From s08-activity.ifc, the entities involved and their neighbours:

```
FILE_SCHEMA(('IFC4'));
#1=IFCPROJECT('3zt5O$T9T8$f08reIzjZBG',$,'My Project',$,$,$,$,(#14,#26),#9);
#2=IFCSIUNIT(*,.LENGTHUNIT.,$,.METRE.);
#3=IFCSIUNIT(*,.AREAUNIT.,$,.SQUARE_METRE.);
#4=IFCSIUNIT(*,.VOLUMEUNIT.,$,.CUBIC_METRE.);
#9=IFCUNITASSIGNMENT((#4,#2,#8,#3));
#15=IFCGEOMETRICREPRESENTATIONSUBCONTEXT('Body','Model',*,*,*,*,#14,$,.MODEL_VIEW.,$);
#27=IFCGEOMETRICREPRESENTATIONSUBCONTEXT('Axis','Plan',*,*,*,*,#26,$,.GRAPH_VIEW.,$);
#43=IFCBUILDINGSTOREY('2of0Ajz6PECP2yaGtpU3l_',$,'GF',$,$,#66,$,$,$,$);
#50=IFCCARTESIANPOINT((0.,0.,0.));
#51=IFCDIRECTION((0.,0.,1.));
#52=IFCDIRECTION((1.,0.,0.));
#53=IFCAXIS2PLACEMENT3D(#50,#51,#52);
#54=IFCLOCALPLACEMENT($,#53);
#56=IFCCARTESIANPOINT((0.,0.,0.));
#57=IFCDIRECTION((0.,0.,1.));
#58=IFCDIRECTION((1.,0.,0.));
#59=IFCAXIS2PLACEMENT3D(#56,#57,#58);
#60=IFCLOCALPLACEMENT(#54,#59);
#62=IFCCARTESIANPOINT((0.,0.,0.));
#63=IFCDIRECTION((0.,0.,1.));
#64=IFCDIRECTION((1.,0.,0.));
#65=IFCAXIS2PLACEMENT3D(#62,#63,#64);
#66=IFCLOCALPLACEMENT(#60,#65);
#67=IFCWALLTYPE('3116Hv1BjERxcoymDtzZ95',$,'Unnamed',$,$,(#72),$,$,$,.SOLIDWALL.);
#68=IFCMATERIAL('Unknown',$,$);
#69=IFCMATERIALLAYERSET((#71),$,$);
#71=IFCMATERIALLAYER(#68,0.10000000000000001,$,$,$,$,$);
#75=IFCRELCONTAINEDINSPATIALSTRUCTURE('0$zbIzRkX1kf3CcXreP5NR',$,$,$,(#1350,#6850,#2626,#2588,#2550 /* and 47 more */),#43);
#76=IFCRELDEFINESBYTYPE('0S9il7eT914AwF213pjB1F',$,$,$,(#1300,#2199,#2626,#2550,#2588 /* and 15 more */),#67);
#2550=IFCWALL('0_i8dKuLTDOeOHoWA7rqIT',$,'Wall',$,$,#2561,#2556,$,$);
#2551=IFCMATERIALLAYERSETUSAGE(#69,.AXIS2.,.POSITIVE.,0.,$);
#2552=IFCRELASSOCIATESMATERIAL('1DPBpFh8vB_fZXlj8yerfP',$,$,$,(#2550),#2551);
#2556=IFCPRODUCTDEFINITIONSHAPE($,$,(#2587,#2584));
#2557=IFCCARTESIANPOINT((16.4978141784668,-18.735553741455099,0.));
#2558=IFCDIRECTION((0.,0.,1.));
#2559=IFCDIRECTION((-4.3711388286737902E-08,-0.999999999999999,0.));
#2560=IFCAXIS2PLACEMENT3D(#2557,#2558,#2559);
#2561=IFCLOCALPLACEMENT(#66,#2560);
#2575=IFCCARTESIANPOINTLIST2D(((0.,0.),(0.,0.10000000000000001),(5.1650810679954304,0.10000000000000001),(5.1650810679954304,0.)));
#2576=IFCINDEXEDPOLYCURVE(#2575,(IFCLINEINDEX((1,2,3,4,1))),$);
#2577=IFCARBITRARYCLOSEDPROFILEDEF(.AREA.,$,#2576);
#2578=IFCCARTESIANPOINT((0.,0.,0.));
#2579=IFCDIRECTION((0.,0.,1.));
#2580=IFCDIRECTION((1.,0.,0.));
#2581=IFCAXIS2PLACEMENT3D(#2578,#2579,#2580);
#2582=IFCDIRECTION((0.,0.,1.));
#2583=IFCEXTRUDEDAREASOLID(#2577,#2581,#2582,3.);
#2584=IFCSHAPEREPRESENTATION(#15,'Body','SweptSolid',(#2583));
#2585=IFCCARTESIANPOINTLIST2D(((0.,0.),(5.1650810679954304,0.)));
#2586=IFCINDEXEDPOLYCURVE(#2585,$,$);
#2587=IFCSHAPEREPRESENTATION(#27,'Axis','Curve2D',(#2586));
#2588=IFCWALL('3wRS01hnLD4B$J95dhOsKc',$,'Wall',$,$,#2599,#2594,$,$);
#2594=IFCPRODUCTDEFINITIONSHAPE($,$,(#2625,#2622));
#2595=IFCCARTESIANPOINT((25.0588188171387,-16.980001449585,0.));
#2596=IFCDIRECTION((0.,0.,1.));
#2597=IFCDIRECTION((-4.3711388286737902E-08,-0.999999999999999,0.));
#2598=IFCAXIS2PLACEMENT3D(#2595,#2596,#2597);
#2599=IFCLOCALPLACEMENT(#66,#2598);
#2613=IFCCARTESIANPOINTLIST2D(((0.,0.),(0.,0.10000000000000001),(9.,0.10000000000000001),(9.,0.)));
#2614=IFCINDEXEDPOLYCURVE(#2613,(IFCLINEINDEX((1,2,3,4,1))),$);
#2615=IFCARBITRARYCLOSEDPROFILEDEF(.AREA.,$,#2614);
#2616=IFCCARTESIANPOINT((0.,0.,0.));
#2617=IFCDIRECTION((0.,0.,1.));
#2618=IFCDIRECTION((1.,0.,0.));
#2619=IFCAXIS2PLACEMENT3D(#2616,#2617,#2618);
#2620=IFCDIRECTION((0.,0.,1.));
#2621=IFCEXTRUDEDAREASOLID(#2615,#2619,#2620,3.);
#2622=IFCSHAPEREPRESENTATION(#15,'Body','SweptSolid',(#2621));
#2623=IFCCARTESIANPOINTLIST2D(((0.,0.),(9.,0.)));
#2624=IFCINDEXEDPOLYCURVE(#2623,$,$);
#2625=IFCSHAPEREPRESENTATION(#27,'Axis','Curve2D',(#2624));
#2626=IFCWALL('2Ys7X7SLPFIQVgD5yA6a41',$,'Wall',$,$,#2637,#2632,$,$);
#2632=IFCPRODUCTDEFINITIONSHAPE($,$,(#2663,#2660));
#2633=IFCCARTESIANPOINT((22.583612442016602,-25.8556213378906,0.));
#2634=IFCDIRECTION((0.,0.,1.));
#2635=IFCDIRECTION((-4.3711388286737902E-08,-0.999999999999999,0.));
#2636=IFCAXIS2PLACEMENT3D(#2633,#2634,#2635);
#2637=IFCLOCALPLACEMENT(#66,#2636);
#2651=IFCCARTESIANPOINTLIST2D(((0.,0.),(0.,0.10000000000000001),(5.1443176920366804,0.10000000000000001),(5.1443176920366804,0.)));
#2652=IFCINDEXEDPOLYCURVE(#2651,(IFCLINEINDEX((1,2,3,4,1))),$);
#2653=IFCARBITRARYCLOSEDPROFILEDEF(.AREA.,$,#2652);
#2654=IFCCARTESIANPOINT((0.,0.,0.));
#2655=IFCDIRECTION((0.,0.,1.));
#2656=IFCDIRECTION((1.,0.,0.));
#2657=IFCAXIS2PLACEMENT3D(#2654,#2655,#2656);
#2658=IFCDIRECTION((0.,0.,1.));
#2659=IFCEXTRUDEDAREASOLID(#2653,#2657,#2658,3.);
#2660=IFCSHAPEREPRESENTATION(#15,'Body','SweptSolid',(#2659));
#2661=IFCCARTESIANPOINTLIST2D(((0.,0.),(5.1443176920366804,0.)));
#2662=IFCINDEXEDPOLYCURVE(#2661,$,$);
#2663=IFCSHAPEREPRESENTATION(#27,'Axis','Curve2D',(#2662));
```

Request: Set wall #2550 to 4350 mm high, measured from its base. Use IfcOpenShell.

```python
import ifcopenshell
import ifcopenshell.geom
import ifcopenshell.util.representation
import ifcopenshell.util.shape
import ifcopenshell.util.unit

model = ifcopenshell.open("s08-activity.ifc")
unit_scale = ifcopenshell.util.unit.calculate_unit_scale(model)
settings = ifcopenshell.geom.settings()


def volume(element):
    """Net volume in cubic metres, openings subtracted."""
    shape = ifcopenshell.geom.create_shape(settings, element)
    return ifcopenshell.util.shape.get_volume(shape.geometry)


wall = model.by_guid("0_i8dKuLTDOeOHoWA7rqIT")
before = volume(wall)

body = ifcopenshell.util.representation.get_representation(wall, "Model", "Body")
solid = body.Items[0]
old_height = solid.Depth
solid.Depth = 4.35 / unit_scale
after = volume(wall)

print(f"height {old_height:g} -> {solid.Depth:g}, volume {before:.3f} -> {after:.3f} m3")

model.write("s08-activity_edited.ifc")
```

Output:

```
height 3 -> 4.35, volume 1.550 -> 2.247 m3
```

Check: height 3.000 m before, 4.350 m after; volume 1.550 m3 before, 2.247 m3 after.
